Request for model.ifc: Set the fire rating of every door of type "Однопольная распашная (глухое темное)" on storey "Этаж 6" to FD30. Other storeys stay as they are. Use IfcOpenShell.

First a look at what the model holds.

```python
import ifcopenshell
import ifcopenshell.util.element

model = ifcopenshell.open("model.ifc")
print(model.schema)
storey = next(s for s in model.by_type("IfcBuildingStorey") if s.Name == "Этаж 6")
doors = [e for e in ifcopenshell.util.element.get_decomposition(storey) if e.is_a("IfcDoor")]
seen = {}
for e in doors:
    element_type = ifcopenshell.util.element.get_type(e)
    key = (element_type.Name if element_type != e and element_type else None, ifcopenshell.util.element.get_pset(e, "Pset_DoorCommon", "FireRating"))
    seen[key] = seen.get(key, 0) + 1
for (name, value), count in sorted(seen.items(), key=str):
    print(count, "x", name, "|", value)
```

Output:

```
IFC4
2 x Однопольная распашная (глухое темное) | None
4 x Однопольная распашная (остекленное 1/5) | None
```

```python
import ifcopenshell
import ifcopenshell.api.pset
import ifcopenshell.util.element

model = ifcopenshell.open("model.ifc")

storey = next(s for s in model.by_type("IfcBuildingStorey") if s.Name == "Этаж 6")
doors = [e for e in ifcopenshell.util.element.get_decomposition(storey) if e.is_a("IfcDoor")]

count = 0
for e in doors:
    element_type = ifcopenshell.util.element.get_type(e)
    if element_type in (None, e) or element_type.Name != "Однопольная распашная (глухое темное)":
        continue
    # add_pset returns the element's existing set when there is one.
    pset = ifcopenshell.api.pset.add_pset(model, product=e, name="Pset_DoorCommon")
    ifcopenshell.api.pset.edit_pset(model, pset=pset, properties={"FireRating": "FD30"})
    count += 1

print(count, "doors updated")

model.write("model_v2.ifc")
```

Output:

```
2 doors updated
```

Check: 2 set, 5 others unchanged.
